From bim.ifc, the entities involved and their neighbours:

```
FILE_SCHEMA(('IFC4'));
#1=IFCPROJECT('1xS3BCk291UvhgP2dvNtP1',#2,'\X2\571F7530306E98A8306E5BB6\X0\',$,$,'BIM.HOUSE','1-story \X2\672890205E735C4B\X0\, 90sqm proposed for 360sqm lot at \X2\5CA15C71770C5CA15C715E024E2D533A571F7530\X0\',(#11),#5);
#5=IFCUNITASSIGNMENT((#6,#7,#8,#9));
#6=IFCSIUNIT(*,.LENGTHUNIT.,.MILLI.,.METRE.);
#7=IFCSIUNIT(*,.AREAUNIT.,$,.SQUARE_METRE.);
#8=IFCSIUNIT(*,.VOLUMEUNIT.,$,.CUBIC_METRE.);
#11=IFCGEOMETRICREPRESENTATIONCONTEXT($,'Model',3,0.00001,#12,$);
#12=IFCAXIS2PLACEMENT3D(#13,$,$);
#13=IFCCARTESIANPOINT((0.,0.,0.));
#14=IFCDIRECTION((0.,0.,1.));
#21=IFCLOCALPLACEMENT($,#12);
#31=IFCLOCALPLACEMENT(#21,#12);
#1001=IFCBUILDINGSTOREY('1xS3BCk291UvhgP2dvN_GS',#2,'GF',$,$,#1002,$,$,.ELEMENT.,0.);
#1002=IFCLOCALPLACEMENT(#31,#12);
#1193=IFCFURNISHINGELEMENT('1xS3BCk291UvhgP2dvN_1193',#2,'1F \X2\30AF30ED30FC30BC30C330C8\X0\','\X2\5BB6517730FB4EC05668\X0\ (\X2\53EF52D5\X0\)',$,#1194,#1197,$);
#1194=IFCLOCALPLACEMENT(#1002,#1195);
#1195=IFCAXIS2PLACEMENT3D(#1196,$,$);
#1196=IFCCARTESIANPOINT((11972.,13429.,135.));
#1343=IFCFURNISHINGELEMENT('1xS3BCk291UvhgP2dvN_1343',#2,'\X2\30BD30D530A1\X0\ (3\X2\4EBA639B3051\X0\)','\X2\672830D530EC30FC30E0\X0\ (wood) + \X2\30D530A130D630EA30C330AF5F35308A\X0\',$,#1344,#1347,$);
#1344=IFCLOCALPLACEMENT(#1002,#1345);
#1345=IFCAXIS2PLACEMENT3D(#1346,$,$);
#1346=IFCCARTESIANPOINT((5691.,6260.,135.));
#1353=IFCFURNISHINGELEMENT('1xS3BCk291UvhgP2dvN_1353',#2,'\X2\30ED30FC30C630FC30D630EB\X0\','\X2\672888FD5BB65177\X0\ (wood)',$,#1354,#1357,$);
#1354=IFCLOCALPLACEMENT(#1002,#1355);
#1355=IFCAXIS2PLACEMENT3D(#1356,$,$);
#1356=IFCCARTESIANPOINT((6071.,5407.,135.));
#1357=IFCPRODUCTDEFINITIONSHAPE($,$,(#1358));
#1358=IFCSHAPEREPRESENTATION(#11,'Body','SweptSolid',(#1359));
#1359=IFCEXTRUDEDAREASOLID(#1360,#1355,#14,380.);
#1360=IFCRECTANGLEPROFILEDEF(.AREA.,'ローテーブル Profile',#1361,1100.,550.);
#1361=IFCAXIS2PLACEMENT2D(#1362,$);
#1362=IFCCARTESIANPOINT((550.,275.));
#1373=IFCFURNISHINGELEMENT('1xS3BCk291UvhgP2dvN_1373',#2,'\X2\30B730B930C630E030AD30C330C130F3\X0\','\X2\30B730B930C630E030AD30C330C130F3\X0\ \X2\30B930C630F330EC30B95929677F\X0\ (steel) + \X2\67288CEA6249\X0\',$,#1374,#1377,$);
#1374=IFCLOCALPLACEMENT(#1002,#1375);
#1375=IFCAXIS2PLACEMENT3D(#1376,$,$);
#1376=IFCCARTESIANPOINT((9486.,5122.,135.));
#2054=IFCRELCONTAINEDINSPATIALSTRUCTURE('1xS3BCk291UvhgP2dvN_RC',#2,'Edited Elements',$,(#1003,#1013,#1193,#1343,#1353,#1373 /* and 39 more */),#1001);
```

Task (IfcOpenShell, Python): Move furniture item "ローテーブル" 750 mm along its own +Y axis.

```python
import ifcopenshell
import ifcopenshell.api.geometry
import ifcopenshell.util.placement
import ifcopenshell.util.unit

model = ifcopenshell.open("bim.ifc")
unit_scale = ifcopenshell.util.unit.calculate_unit_scale(model)

item = model.by_guid("1xS3BCk291UvhgP2dvN_1353")
matrix = ifcopenshell.util.placement.get_local_placement(item.ObjectPlacement)
matrix[:3, 3] += matrix[:3, 1] * 0.75 / unit_scale
ifcopenshell.api.geometry.edit_object_placement(model, product=item, matrix=matrix, is_si=False)

print(ifcopenshell.util.placement.get_local_placement(item.ObjectPlacement).round(3) + 0.0)

model.write("bim_updated.ifc")
```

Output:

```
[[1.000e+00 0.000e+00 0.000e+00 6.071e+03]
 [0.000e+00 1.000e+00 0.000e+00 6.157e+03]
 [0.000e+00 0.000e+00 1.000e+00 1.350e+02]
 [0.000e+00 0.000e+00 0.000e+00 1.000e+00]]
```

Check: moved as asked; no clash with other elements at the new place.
